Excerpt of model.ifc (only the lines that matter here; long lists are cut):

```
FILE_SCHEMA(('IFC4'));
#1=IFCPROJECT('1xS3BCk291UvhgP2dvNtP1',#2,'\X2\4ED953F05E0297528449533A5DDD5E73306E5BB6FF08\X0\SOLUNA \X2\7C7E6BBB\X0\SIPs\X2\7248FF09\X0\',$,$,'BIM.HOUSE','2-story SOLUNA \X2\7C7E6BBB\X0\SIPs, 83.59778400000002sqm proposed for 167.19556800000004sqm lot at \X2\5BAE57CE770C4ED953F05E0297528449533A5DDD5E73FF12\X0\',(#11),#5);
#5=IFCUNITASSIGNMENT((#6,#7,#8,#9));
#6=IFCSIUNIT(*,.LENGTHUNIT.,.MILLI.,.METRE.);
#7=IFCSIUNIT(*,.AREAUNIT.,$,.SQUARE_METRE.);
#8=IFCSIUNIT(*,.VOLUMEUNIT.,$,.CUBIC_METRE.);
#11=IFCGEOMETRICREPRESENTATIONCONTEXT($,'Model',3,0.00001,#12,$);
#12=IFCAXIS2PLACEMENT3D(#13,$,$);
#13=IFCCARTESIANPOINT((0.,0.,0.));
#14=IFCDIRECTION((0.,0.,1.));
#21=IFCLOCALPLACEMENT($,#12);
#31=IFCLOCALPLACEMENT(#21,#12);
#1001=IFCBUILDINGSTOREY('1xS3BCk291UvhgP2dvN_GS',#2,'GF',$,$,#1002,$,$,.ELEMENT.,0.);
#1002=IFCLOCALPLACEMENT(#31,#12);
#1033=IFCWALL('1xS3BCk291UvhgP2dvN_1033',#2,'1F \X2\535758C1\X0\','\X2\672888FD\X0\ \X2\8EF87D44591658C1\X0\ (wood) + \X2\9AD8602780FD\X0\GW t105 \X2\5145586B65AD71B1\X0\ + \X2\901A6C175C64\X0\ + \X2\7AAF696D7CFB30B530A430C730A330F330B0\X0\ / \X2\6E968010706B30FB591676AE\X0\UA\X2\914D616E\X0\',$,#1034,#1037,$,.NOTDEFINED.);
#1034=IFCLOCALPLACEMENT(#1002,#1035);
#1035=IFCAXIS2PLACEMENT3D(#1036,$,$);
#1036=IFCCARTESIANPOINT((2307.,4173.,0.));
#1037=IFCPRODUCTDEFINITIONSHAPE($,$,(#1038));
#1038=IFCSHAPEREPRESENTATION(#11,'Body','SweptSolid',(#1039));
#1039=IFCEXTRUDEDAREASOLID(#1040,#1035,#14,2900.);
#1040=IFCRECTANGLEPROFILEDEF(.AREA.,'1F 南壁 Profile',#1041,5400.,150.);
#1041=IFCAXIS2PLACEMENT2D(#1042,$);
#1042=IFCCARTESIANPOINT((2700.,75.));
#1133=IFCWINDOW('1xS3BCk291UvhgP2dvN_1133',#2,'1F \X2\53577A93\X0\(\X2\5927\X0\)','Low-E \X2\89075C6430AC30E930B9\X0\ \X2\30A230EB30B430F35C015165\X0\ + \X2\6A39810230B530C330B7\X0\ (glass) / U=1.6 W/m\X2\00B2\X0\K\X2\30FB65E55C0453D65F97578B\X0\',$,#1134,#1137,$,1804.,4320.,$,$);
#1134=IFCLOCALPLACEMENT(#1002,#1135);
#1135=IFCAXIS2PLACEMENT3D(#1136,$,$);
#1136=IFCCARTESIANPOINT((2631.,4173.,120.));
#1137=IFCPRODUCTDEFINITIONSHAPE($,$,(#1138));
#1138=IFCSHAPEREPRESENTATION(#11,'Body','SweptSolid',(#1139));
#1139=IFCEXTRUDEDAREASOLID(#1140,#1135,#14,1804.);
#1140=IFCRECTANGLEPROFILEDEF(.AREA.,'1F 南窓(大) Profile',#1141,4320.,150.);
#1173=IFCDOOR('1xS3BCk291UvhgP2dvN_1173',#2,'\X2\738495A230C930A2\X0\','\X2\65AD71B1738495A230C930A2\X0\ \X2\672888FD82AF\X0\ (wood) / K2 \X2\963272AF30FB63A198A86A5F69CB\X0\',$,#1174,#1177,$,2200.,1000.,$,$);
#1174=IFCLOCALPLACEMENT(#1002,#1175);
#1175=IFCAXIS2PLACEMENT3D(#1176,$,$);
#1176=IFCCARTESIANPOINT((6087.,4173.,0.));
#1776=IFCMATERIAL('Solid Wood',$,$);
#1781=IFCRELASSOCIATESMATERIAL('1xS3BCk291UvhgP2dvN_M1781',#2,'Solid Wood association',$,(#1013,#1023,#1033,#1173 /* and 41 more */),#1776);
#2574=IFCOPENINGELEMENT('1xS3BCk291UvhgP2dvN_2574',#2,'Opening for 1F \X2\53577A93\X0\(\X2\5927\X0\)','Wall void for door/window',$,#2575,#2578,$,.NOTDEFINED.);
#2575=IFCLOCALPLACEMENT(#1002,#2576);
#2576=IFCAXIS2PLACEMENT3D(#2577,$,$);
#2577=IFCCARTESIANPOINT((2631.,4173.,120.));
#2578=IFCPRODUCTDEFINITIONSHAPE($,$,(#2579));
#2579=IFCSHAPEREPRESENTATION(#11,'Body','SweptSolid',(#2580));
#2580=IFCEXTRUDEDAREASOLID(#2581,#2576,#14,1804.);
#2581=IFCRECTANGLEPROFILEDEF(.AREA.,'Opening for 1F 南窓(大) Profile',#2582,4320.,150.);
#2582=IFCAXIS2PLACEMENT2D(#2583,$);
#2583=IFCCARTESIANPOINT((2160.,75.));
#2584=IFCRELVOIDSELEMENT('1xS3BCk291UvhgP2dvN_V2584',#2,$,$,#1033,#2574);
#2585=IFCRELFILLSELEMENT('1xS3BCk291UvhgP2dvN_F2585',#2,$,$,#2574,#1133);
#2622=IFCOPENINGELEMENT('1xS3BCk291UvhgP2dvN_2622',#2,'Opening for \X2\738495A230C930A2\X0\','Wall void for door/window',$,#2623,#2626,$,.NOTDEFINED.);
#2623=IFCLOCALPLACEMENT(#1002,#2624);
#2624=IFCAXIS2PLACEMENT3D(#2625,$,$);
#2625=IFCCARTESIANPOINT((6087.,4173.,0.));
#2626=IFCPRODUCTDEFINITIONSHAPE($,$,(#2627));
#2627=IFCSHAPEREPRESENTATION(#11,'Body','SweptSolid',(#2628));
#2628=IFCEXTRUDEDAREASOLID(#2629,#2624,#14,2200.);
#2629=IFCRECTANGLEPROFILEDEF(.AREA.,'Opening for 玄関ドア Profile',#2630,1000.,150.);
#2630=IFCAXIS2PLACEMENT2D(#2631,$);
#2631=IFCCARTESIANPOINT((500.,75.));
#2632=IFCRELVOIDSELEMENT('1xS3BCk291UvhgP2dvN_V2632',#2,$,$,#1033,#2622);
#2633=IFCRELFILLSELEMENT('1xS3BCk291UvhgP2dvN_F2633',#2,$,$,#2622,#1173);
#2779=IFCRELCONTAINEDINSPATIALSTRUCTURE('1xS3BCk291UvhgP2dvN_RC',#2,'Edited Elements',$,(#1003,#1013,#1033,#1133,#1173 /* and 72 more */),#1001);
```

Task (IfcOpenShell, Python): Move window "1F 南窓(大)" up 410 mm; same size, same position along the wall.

```python
import numpy as np
import ifcopenshell
import ifcopenshell.api.geometry
import ifcopenshell.util.placement
import ifcopenshell.util.unit

model = ifcopenshell.open("model.ifc")
unit_scale = ifcopenshell.util.unit.calculate_unit_scale(model)

window = model.by_guid("1xS3BCk291UvhgP2dvN_1133")
opening = window.FillsVoids[0].RelatingOpeningElement
dz = 0.41 / unit_scale

shift = np.array([0.0, 0.0, dz])
# The window is not placed relative to its opening, so move both.
for product in (opening, window):
    matrix = ifcopenshell.util.placement.get_local_placement(product.ObjectPlacement)
    matrix[:3, 3] += shift
    ifcopenshell.api.geometry.edit_object_placement(model, product=product, matrix=matrix, is_si=False)

print(f"moved by {dz * unit_scale:+.3f} m")

model.write("model_updated.ifc")
```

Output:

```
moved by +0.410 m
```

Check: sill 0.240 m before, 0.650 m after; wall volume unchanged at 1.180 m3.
